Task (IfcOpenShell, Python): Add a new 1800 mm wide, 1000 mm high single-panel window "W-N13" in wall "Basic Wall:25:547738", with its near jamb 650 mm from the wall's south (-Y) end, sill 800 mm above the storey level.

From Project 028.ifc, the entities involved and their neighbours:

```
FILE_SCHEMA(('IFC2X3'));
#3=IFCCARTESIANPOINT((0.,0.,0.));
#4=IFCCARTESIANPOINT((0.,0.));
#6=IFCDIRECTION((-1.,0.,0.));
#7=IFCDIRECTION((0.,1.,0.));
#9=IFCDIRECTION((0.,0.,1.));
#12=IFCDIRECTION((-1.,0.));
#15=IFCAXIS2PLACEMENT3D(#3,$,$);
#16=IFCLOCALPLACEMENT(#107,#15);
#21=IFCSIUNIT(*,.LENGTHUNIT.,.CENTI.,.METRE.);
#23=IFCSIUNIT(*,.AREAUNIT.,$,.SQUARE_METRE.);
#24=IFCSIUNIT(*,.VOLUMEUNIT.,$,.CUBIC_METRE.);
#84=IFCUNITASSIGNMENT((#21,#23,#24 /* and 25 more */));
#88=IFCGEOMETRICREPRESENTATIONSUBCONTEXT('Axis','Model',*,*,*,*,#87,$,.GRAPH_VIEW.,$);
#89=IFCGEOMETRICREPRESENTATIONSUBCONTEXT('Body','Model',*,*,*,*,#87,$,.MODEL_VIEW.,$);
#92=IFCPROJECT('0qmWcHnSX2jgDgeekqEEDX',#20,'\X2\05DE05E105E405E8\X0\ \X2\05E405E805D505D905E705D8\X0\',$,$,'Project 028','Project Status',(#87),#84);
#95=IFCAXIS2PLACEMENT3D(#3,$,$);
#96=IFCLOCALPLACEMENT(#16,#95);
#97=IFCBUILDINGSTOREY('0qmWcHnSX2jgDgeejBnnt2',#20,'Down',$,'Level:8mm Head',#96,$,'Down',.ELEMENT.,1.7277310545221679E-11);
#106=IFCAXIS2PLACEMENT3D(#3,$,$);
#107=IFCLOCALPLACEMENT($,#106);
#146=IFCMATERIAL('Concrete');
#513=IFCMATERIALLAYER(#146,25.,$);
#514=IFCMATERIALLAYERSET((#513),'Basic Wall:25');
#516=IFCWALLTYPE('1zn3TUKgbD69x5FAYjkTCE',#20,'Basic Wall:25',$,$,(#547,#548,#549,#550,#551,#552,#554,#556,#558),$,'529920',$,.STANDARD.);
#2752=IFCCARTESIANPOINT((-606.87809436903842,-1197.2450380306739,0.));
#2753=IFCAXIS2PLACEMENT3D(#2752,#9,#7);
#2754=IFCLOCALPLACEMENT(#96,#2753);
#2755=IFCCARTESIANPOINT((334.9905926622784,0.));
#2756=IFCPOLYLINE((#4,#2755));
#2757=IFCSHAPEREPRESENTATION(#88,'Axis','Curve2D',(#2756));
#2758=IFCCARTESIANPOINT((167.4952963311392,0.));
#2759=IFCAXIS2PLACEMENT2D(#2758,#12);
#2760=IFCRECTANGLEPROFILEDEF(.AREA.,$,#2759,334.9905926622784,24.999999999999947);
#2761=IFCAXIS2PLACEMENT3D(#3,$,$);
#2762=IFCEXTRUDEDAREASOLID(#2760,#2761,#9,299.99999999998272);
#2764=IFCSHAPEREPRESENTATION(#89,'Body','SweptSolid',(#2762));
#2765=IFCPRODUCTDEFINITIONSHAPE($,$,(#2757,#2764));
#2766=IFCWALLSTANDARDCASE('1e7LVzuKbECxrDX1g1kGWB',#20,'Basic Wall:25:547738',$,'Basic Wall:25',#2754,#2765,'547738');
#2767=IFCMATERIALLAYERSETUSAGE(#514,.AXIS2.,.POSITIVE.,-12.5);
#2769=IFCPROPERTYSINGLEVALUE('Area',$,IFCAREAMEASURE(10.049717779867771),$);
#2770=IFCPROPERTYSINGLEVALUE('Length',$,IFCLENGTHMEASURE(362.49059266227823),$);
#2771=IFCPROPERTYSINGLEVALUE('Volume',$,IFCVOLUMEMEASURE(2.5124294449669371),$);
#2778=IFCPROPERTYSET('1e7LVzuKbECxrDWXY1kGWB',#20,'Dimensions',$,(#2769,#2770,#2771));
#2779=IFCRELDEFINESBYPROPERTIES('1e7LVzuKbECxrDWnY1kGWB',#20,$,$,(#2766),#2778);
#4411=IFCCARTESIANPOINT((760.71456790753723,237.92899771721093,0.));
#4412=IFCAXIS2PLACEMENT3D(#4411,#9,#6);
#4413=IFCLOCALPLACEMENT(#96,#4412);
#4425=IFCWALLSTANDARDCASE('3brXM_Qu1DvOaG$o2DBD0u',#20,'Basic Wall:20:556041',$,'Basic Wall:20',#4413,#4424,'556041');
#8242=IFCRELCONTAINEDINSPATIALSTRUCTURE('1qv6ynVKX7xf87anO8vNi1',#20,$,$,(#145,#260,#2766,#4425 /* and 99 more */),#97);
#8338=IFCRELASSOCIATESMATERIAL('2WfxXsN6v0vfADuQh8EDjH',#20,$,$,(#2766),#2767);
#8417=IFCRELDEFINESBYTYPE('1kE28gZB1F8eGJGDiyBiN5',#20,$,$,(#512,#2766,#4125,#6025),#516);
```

```python
import numpy as np
import ifcopenshell
import ifcopenshell.api.feature
import ifcopenshell.api.geometry
import ifcopenshell.api.pset
import ifcopenshell.api.root
import ifcopenshell.api.spatial
import ifcopenshell.api.type
import ifcopenshell.geom
import ifcopenshell.util.element
import ifcopenshell.util.placement
import ifcopenshell.util.representation
import ifcopenshell.util.shape
import ifcopenshell.util.unit

model = ifcopenshell.open("Project 028.ifc")
unit_scale = ifcopenshell.util.unit.calculate_unit_scale(model)
area_scale = ifcopenshell.util.unit.calculate_unit_scale(model, "AREAUNIT")
volume_scale = ifcopenshell.util.unit.calculate_unit_scale(model, "VOLUMEUNIT")
settings = ifcopenshell.geom.settings()


def volume(element):
    """Net volume in cubic metres, openings subtracted."""
    shape = ifcopenshell.geom.create_shape(settings, element)
    return ifcopenshell.util.shape.get_volume(shape.geometry)


wall = model.by_id(2766)
storey = ifcopenshell.util.element.get_container(wall, ifc_class="IfcBuildingStorey")
context = ifcopenshell.util.representation.get_context(model, "Model", "Body", "MODEL_VIEW")
before = volume(wall)

width, height, from_end, sill = 1.8, 1, 0.65, 0.8  # metres

# The wall runs along its own X axis, and the end named is its -X end.
wall_shape = ifcopenshell.geom.create_shape(settings, wall)
x, y, z = ifcopenshell.util.shape.get_vertices(wall_shape.geometry).T
start = x.min() + from_end
face, thickness = float(y.min()), float(y.max() - y.min())
wall_matrix = ifcopenshell.util.placement.get_local_placement(wall.ObjectPlacement)
level = ifcopenshell.util.placement.get_local_placement(storey.ObjectPlacement)[2, 3]


def in_wall(x, y):
    """Placement at x, y metres in the wall's axes, at sill height."""
    matrix = wall_matrix.copy()
    matrix[:, 3] = wall_matrix @ np.array([x / unit_scale, y / unit_scale, 0.0, 1.0])
    matrix[2, 3] = level + sill / unit_scale
    return matrix


# Opening: a box that overshoots both wall faces by 50 mm.
opening = ifcopenshell.api.root.create_entity(model, ifc_class="IfcOpeningElement")
box = ifcopenshell.api.geometry.add_wall_representation(
    model, context=context, length=width, height=height, thickness=thickness + 0.1
)
ifcopenshell.api.geometry.assign_representation(model, product=opening, representation=box)
ifcopenshell.api.geometry.edit_object_placement(model, product=opening, matrix=in_wall(start, face - 0.05), is_si=False)
ifcopenshell.api.feature.add_feature(model, feature=opening, element=wall)

window = ifcopenshell.api.root.create_entity(model, ifc_class="IfcWindow", name="W-N13")
window.OverallWidth, window.OverallHeight = width / unit_scale, height / unit_scale
body = ifcopenshell.api.geometry.add_window_representation(
    model,
    context=context,
    overall_width=window.OverallWidth,
    overall_height=window.OverallHeight,
    partition_type="SINGLE_PANEL",
)
ifcopenshell.api.geometry.assign_representation(model, product=window, representation=body)
ifcopenshell.api.spatial.assign_container(model, products=[window], relating_structure=storey)
fills = ifcopenshell.api.feature.add_filling(model, opening=opening, element=window)
fills.OwnerHistory = window.OwnerHistory  # required in IFC2X3

# IFC2X3 keeps the operation on the window style.
style = ifcopenshell.api.root.create_entity(model, ifc_class="IfcWindowStyle", name="W-N13")
style.OperationType, style.ConstructionType = "SINGLE_PANEL", "NOTDEFINED"
style.ParameterTakesPrecedence = style.Sizeable = False
ifcopenshell.api.type.assign_type(model, related_objects=[window], relating_type=style)

# Centre the window in the wall's thickness.
ifcopenshell.api.geometry.edit_object_placement(model, product=window, matrix=in_wall(start, face), is_si=False)
window_shape = ifcopenshell.geom.create_shape(settings, window)
depth = ifcopenshell.util.shape.get_vertices(window_shape.geometry)[:, 1]
offset = face + thickness / 2 - (depth.min() + depth.max()) / 2
ifcopenshell.api.geometry.edit_object_placement(model, product=window, matrix=in_wall(start, offset), is_si=False)

after = volume(wall)

# Update the wall's stored quantities.
pset = model.by_id(ifcopenshell.util.element.get_pset(wall, "Dimensions", should_inherit=False)["id"])
ifcopenshell.api.pset.edit_pset(model, pset=pset, properties={
    "Area": model.create_entity("IfcAreaMeasure", after / thickness / area_scale),
    "Volume": model.create_entity("IfcVolumeMeasure", after / volume_scale),
})

print(f"wall volume {before:.3f} -> {after:.3f} m3")

model.write("Project 028_edited.ifc")
```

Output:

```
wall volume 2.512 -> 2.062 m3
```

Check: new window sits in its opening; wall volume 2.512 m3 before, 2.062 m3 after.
